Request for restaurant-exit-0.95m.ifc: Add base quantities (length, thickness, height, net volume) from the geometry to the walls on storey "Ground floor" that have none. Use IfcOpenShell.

First a look at what the model holds.

```python
import ifcopenshell
import ifcopenshell.util.element
import ifcopenshell.util.unit

model = ifcopenshell.open("restaurant-exit-0.95m.ifc")
print(model.schema)
for unit_type in ("LENGTHUNIT", "AREAUNIT", "VOLUMEUNIT"):
    print(unit_type, ifcopenshell.util.unit.calculate_unit_scale(model, unit_type))
storey = next(s for s in model.by_type("IfcBuildingStorey") if s.Name == "Ground floor")
walls = [e for e in ifcopenshell.util.element.get_decomposition(storey) if e.is_a("IfcWall")]
for e in sorted(walls, key=lambda e: e.id()):
    print(e.id(), e.is_a(), e.Name, list(ifcopenshell.util.element.get_psets(e, qtos_only=True)), sep=" | ")
```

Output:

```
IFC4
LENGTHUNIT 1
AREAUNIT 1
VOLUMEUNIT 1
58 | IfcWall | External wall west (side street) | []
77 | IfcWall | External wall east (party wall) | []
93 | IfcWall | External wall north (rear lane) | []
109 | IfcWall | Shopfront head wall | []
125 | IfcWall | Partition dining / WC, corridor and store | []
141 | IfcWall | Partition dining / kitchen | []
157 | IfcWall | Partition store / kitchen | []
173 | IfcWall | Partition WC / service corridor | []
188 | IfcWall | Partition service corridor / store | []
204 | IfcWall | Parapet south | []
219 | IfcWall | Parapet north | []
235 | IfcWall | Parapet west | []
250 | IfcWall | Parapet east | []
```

```python
import ifcopenshell
import ifcopenshell.api.pset
import ifcopenshell.geom
import ifcopenshell.util.element
import ifcopenshell.util.shape
import ifcopenshell.util.unit

model = ifcopenshell.open("restaurant-exit-0.95m.ifc")
unit_scale = ifcopenshell.util.unit.calculate_unit_scale(model)
volume_scale = ifcopenshell.util.unit.calculate_unit_scale(model, "VOLUMEUNIT")
settings = ifcopenshell.geom.settings()

storey = next(s for s in model.by_type("IfcBuildingStorey") if s.Name == "Ground floor")
walls = [e for e in ifcopenshell.util.element.get_decomposition(storey) if e.is_a("IfcWall")]

for e in sorted(walls, key=lambda e: e.id()):
    if ifcopenshell.util.element.get_psets(e, qtos_only=True, should_inherit=False):
        continue
    # Geometry comes back in metres, in the element's own axes.
    shape = ifcopenshell.geom.create_shape(settings, e)
    values = {
        "Length": ifcopenshell.util.shape.get_x(shape.geometry) / unit_scale,
        "Width": ifcopenshell.util.shape.get_y(shape.geometry) / unit_scale,
        "Height": ifcopenshell.util.shape.get_z(shape.geometry) / unit_scale,
        "NetVolume": ifcopenshell.util.shape.get_volume(shape.geometry) / volume_scale,
    }
    qto = ifcopenshell.api.pset.add_qto(model, product=e, name="Qto_WallBaseQuantities")
    ifcopenshell.api.pset.edit_qto(model, qto=qto, properties=values)
    print(e.id(), {k: round(v, 3) for k, v in values.items()})

model.write("restaurant-exit-0.95m_rev.ifc")
```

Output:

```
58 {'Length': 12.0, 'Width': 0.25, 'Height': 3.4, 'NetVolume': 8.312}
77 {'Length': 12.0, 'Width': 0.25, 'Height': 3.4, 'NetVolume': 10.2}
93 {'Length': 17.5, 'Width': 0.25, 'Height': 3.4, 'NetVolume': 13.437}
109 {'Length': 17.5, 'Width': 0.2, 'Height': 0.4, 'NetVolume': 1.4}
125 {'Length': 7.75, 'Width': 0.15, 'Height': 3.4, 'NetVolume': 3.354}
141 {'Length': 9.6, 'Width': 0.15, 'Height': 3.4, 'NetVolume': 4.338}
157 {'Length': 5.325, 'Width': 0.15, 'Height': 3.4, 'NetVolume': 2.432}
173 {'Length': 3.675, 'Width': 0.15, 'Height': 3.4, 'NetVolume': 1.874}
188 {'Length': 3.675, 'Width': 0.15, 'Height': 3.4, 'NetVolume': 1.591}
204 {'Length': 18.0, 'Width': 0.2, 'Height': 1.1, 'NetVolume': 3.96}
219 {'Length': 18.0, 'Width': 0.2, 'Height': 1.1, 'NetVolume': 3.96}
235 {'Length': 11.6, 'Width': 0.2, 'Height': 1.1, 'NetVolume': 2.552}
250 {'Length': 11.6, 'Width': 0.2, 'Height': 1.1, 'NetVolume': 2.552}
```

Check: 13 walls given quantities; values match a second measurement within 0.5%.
